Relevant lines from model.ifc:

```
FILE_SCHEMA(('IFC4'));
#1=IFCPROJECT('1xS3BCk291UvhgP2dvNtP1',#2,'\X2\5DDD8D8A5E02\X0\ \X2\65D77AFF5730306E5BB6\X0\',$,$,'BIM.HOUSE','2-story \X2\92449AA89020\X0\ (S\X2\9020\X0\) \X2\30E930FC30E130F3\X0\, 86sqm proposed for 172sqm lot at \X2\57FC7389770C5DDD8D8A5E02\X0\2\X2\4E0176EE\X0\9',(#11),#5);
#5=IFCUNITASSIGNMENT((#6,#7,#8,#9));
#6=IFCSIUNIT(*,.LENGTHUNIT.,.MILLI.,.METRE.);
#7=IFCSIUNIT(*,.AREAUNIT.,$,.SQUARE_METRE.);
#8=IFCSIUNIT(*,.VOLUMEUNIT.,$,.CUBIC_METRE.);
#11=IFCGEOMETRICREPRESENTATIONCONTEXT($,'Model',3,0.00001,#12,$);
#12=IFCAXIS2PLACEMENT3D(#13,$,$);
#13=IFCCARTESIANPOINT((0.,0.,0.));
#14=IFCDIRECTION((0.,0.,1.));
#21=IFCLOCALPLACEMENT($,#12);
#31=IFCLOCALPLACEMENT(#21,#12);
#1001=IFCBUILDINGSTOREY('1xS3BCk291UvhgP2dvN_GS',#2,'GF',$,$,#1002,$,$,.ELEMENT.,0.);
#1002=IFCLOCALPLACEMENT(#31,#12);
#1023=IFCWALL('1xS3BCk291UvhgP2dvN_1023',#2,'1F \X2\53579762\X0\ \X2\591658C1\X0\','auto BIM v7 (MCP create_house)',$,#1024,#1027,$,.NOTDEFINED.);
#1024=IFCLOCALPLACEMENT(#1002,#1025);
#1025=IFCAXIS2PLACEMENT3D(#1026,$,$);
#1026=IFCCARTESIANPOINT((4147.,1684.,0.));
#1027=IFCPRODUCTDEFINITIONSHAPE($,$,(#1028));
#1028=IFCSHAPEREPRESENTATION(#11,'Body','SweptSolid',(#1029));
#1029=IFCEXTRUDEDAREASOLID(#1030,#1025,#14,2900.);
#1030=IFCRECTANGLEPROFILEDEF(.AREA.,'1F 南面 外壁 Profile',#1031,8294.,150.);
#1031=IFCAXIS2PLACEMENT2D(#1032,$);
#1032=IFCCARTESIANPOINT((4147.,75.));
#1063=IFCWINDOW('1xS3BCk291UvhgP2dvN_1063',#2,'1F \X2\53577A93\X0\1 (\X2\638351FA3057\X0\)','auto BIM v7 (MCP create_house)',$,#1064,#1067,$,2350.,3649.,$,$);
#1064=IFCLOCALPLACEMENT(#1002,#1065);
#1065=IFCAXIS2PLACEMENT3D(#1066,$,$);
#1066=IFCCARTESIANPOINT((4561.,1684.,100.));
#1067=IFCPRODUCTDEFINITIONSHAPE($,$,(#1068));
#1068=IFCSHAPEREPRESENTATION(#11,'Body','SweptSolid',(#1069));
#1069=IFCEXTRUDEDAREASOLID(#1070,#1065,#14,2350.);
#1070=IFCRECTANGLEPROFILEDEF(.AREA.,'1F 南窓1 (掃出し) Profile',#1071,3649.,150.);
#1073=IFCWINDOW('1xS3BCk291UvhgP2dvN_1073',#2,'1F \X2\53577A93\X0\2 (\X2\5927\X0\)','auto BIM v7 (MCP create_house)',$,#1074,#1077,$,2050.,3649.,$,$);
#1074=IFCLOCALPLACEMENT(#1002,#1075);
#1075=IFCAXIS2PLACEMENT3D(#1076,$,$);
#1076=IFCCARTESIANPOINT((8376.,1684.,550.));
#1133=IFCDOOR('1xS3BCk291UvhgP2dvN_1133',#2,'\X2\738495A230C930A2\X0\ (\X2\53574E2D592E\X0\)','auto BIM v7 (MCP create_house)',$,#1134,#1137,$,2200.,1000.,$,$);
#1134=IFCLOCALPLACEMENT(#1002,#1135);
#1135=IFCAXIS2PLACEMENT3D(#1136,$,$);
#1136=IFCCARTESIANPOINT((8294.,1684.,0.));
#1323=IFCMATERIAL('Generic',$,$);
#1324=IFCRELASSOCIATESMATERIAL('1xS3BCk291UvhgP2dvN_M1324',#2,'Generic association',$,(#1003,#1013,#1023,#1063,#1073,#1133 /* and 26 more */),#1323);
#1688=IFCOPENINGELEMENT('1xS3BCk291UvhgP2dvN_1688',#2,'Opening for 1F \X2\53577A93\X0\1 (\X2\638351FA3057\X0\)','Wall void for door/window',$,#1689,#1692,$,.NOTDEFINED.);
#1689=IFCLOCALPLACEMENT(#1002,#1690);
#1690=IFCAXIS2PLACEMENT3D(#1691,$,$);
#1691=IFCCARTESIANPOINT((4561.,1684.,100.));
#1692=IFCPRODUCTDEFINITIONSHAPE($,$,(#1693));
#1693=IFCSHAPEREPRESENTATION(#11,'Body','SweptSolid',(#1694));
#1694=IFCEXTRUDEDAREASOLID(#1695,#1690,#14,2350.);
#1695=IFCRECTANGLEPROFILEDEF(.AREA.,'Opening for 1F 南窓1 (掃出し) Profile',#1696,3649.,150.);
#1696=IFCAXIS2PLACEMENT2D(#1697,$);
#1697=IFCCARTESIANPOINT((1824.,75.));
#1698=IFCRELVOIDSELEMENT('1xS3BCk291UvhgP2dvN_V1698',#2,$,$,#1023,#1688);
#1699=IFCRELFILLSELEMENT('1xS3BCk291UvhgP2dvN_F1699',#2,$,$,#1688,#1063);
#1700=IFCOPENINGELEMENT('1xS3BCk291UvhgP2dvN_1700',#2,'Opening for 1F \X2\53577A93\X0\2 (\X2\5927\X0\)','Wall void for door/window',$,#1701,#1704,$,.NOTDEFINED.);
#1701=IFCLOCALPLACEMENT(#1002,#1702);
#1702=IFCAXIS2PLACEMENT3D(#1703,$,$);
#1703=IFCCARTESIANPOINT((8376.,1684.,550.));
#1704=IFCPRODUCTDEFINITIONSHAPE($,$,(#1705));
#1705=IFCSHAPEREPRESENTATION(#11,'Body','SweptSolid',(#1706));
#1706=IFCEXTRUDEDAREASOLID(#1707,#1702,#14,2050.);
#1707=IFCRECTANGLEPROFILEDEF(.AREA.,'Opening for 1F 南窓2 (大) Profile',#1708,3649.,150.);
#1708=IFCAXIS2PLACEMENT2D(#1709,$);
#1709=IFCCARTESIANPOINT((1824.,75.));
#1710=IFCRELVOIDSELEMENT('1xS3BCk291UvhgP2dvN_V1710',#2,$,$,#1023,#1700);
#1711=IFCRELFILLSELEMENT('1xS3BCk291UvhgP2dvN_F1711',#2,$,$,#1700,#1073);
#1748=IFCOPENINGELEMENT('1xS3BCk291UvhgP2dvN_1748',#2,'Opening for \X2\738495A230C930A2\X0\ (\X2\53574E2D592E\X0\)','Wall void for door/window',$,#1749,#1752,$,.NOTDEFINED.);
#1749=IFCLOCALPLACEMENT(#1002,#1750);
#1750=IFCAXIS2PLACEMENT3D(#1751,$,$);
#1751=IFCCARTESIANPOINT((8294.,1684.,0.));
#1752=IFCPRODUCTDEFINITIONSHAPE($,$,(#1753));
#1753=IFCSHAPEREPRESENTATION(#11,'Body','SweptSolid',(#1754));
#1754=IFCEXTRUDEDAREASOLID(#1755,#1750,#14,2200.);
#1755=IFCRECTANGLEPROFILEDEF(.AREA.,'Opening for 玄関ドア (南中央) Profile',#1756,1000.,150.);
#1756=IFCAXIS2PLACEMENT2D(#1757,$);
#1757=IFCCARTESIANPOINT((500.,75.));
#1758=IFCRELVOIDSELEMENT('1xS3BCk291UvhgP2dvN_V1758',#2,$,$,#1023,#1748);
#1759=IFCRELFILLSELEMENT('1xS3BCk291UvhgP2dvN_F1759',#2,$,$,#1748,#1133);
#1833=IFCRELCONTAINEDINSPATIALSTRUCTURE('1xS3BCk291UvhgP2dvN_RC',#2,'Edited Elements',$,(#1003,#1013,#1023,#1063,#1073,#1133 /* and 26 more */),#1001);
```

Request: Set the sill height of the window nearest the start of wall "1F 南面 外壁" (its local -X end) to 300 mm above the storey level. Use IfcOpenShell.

```python
import numpy as np
import ifcopenshell
import ifcopenshell.api.geometry
import ifcopenshell.geom
import ifcopenshell.util.element
import ifcopenshell.util.placement
import ifcopenshell.util.shape
import ifcopenshell.util.unit

model = ifcopenshell.open("model.ifc")
unit_scale = ifcopenshell.util.unit.calculate_unit_scale(model)

window = model.by_guid("1xS3BCk291UvhgP2dvN_1063")
opening = window.FillsVoids[0].RelatingOpeningElement
storey = ifcopenshell.util.element.get_container(window, ifc_class="IfcBuildingStorey")
level = ifcopenshell.util.placement.get_local_placement(storey.ObjectPlacement)[2, 3]

# The opening's origin need not be at the sill, so measure its lowest point.
shape = ifcopenshell.geom.create_shape(ifcopenshell.geom.settings(), opening)
bottom = ifcopenshell.util.shape.get_shape_bottom_elevation(shape, shape.geometry) / unit_scale
dz = level + 0.3 / unit_scale - bottom

shift = np.array([0.0, 0.0, dz])
# The window is not placed relative to its opening, so move both.
for product in (opening, window):
    matrix = ifcopenshell.util.placement.get_local_placement(product.ObjectPlacement)
    matrix[:3, 3] += shift
    ifcopenshell.api.geometry.edit_object_placement(model, product=product, matrix=matrix, is_si=False)

print(f"moved by {dz * unit_scale:+.3f} m")

model.write("model_edited.ifc")
```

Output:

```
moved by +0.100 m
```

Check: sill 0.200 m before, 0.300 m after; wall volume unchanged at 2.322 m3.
